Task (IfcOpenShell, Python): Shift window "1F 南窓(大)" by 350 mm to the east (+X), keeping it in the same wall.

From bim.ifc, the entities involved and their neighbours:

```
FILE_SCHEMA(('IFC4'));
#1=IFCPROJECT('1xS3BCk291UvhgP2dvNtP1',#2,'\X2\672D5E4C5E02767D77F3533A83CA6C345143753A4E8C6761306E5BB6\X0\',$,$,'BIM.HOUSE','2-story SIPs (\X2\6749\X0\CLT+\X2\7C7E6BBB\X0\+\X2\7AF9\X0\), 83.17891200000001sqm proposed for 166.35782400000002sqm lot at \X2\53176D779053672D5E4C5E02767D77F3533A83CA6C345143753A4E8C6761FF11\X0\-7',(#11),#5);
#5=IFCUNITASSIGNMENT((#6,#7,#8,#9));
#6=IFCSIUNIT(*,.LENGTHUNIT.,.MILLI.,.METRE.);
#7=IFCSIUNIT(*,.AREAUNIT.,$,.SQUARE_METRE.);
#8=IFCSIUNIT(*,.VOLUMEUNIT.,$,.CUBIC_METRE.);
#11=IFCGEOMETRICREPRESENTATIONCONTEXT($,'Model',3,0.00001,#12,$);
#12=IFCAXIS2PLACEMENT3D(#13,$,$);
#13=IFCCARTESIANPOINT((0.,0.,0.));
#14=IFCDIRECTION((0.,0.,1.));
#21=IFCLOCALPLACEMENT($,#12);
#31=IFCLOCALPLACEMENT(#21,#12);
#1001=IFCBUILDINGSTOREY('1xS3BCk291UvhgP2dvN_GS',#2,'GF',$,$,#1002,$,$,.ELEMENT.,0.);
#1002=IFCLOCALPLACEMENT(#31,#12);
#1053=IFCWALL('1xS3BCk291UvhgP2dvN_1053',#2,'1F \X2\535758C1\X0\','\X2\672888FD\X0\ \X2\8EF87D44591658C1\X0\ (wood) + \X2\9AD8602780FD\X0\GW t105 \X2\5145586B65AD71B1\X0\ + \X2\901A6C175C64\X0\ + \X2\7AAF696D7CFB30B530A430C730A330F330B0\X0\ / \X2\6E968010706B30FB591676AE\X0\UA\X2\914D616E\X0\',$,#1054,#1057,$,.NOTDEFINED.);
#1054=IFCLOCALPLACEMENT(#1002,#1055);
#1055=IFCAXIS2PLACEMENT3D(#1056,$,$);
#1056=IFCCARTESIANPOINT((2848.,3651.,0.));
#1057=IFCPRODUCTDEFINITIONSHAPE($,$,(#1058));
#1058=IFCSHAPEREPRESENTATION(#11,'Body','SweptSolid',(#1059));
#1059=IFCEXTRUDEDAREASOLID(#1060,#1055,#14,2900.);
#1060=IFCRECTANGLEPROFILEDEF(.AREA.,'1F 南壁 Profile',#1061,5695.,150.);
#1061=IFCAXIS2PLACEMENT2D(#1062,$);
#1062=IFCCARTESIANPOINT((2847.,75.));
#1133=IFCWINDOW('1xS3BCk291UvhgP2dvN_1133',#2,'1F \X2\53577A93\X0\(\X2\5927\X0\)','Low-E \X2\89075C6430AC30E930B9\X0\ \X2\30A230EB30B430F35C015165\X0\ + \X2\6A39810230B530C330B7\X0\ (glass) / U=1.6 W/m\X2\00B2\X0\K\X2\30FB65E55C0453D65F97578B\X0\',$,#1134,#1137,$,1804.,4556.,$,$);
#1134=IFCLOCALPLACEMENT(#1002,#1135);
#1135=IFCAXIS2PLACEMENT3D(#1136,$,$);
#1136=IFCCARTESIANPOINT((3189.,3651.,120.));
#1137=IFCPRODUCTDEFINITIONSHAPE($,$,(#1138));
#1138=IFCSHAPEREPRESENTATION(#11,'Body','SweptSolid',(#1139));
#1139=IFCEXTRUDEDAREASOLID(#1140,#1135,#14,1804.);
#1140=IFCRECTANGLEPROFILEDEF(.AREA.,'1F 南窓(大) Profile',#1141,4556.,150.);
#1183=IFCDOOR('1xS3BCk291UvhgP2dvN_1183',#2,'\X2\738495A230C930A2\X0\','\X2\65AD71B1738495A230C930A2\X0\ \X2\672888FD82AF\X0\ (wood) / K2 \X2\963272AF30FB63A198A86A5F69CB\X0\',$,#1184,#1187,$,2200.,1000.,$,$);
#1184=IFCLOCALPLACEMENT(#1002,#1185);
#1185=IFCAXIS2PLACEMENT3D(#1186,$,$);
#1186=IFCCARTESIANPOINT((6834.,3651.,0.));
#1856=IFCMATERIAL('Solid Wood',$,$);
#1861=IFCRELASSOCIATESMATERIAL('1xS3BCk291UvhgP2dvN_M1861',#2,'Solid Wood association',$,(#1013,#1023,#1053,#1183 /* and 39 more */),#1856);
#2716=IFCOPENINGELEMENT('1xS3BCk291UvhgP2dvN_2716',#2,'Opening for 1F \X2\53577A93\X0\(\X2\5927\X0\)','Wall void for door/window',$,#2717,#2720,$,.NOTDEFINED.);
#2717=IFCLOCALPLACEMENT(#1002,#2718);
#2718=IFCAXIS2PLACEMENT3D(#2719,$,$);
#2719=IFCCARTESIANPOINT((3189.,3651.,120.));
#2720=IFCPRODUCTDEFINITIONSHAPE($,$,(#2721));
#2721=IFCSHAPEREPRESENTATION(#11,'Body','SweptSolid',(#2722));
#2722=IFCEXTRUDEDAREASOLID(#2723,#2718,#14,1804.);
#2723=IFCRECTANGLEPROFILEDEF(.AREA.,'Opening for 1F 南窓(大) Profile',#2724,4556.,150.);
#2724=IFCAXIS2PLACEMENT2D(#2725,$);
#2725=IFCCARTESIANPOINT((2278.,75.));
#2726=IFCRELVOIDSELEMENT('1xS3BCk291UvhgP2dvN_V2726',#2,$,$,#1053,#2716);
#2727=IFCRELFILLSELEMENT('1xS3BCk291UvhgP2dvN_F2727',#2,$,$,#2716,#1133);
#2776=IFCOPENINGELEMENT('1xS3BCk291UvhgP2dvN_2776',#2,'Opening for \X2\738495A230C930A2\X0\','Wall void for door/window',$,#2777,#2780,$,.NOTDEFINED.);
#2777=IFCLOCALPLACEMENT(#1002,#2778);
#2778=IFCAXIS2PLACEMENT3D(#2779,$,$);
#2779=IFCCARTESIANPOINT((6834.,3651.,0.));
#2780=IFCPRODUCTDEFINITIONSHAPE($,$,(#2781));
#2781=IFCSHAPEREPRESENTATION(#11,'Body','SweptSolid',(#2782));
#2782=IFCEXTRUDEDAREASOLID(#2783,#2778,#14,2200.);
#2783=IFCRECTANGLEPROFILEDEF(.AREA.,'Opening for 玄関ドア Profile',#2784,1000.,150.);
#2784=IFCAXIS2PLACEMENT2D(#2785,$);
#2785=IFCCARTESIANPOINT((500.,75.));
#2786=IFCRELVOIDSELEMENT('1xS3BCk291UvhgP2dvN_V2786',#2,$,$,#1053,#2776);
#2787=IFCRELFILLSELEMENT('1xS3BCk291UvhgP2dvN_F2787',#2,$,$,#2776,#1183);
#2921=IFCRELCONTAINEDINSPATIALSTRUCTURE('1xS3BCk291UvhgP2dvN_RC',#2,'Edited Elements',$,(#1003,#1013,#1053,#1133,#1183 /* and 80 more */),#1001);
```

```python
import ifcopenshell
import ifcopenshell.api.geometry
import ifcopenshell.util.placement

model = ifcopenshell.open("bim.ifc")

window = model.by_guid("1xS3BCk291UvhgP2dvN_1133")
opening = window.FillsVoids[0].RelatingOpeningElement
wall = opening.VoidsElements[0].RelatingBuildingElement

wall_matrix = ifcopenshell.util.placement.get_local_placement(wall.ObjectPlacement)
shift = wall_matrix[:3, 0] * 350.0
before = ifcopenshell.util.placement.get_local_placement(window.ObjectPlacement)[:3, 3].copy()

# The window is not placed relative to its opening, so move both.
for product in (opening, window):
    matrix = ifcopenshell.util.placement.get_local_placement(product.ObjectPlacement)
    matrix[:3, 3] += shift
    ifcopenshell.api.geometry.edit_object_placement(model, product=product, matrix=matrix, is_si=False)

after = ifcopenshell.util.placement.get_local_placement(window.ObjectPlacement)[:3, 3]
print("window moved by", (after - before).round(3) + 0.0)

model.write("bim_v2.ifc")
```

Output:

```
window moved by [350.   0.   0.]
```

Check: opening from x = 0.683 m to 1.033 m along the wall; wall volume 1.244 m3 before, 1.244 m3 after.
